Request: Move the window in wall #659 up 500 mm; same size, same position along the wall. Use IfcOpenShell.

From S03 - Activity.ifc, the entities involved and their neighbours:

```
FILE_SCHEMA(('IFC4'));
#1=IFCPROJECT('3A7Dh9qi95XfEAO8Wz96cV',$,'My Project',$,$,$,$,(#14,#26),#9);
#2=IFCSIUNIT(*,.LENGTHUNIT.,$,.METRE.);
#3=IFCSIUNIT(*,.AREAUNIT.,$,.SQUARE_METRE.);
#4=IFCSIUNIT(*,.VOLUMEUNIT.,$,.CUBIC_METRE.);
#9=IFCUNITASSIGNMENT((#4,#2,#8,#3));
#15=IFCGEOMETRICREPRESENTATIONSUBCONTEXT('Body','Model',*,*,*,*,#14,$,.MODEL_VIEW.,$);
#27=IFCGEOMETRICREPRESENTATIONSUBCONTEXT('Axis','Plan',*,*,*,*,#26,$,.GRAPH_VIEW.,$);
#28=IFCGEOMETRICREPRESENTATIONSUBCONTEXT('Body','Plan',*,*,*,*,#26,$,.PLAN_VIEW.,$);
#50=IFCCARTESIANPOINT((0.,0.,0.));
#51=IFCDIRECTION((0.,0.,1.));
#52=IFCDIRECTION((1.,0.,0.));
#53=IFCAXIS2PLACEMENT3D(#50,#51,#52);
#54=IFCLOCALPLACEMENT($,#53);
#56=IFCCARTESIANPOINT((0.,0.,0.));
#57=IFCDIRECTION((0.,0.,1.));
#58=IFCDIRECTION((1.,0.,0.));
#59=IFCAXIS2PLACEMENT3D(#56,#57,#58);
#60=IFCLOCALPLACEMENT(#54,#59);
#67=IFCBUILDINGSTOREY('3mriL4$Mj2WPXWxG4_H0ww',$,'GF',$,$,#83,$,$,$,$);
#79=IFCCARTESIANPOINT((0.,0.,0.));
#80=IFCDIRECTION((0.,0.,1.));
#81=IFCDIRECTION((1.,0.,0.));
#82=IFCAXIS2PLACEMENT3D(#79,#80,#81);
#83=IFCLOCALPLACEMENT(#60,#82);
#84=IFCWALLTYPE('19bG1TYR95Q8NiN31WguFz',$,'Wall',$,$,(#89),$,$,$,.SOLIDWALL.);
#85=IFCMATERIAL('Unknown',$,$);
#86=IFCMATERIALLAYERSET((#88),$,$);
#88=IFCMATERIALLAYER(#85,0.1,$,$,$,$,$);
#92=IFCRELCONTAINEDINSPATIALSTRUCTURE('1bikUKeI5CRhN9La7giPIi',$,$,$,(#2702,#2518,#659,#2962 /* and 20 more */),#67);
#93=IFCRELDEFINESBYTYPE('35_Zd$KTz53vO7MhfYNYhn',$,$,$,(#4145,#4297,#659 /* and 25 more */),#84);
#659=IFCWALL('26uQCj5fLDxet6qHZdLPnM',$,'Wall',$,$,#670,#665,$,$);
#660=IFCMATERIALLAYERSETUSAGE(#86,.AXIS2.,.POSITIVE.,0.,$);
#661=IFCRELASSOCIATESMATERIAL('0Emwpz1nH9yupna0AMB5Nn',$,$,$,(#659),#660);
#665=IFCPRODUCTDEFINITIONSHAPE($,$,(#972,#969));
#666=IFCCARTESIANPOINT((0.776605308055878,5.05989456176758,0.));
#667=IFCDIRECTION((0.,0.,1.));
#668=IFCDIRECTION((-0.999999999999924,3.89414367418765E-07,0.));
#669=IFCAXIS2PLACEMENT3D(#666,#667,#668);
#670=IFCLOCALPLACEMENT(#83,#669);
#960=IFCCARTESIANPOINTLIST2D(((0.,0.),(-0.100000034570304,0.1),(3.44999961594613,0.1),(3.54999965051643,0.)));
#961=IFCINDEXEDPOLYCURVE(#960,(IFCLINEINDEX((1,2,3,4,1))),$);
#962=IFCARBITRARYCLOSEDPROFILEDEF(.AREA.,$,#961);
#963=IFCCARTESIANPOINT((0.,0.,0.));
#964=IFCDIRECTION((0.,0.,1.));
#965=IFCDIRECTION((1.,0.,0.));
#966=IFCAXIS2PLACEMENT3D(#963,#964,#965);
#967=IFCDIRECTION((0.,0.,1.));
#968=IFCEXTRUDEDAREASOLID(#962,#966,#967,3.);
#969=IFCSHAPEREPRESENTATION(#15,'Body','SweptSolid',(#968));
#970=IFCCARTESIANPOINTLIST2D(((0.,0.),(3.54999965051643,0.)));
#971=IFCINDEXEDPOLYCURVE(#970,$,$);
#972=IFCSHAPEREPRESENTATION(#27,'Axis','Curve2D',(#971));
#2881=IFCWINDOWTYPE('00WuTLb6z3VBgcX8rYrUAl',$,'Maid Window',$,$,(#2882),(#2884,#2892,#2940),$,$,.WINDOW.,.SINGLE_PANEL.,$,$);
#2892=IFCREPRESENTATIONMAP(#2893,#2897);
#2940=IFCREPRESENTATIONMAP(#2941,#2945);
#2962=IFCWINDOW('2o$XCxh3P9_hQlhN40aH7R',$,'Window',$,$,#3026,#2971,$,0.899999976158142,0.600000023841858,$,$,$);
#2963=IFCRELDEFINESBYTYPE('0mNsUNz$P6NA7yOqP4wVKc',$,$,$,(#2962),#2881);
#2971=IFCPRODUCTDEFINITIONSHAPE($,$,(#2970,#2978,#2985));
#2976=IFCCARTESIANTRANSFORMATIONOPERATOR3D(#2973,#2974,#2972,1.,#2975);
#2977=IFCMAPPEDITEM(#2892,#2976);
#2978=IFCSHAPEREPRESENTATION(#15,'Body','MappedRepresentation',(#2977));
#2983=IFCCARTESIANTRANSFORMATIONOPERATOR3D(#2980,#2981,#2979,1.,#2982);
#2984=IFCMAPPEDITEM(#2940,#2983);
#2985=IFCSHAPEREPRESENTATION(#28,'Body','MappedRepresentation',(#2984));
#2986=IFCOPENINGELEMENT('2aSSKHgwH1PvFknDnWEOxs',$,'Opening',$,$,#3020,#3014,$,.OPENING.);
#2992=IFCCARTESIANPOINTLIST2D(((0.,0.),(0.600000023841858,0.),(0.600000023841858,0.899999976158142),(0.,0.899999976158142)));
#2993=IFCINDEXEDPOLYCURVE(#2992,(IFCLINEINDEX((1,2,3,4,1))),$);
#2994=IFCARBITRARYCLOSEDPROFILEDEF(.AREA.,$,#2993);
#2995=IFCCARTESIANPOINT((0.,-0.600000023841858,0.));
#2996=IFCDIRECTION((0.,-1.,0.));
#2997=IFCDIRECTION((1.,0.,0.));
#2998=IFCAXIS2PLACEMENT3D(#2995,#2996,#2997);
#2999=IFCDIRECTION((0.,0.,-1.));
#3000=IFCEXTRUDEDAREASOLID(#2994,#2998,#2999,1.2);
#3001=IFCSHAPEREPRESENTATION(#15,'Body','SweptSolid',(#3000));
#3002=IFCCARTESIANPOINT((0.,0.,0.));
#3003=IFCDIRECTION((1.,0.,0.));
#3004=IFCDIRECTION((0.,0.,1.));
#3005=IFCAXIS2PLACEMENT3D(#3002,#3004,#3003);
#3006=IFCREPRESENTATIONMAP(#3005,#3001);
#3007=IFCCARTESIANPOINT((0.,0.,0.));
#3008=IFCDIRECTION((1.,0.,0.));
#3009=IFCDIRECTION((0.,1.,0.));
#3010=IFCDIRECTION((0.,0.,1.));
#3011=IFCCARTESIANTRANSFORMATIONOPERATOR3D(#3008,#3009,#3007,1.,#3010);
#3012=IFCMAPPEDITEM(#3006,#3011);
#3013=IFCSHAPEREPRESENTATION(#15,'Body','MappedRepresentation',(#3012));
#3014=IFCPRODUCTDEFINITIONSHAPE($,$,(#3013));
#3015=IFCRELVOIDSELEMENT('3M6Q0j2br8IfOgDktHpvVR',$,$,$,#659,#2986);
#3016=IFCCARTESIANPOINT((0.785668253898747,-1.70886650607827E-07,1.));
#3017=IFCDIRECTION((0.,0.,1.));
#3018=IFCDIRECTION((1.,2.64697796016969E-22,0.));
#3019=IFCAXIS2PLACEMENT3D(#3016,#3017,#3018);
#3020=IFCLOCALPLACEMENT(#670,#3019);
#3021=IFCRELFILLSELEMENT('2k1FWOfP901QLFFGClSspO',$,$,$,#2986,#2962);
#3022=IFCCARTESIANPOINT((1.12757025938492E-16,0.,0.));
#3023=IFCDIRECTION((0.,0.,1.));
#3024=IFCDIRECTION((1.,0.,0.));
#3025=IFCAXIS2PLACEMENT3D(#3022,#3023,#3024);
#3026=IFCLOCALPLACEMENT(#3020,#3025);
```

```python
import numpy as np
import ifcopenshell
import ifcopenshell.api.geometry
import ifcopenshell.util.placement
import ifcopenshell.util.unit

model = ifcopenshell.open("S03 - Activity.ifc")
unit_scale = ifcopenshell.util.unit.calculate_unit_scale(model)

window = model.by_id(2962)
opening = window.FillsVoids[0].RelatingOpeningElement
dz = 0.5

shift = np.array([0.0, 0.0, dz])
# The window is placed relative to its opening, so it follows when the opening moves.
matrix = ifcopenshell.util.placement.get_local_placement(opening.ObjectPlacement)
matrix[:3, 3] += shift
ifcopenshell.api.geometry.edit_object_placement(
    model, product=opening, matrix=matrix, is_si=False, should_transform_children=True
)

print(f"moved by {dz * unit_scale:+.3f} m")

model.write("S03 - Activity-out.ifc")
```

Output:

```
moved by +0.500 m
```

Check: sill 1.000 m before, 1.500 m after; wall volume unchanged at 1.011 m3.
